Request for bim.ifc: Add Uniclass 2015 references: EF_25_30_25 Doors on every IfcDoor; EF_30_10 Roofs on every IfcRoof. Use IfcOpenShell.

First a look at what the model holds.

```python
import ifcopenshell

model = ifcopenshell.open("bim.ifc")
print(model.schema)
print("classifications:", [c.Name for c in model.by_type("IfcClassification")])
for ifc_class in ("IfcDoor", "IfcRoof", "IfcStair", "IfcWall", "IfcWindow"):
    print(ifc_class, len(model.by_type(ifc_class)))
```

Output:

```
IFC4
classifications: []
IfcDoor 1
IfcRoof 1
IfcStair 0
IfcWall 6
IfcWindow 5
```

```python
import ifcopenshell
import ifcopenshell.api.classification

model = ifcopenshell.open("bim.ifc")

system = ifcopenshell.api.classification.add_classification(model, classification="Uniclass 2015")

codes = {
    "IfcDoor": ("EF_25_30_25", "Doors"),
    "IfcRoof": ("EF_30_10", "Roofs"),
}
for ifc_class, (code, name) in codes.items():
    products = model.by_type(ifc_class)
    ifcopenshell.api.classification.add_reference(
        model, products=products, classification=system, identification=code, name=name
    )
    print(code, len(products))

model.write("bim_edited.ifc")
```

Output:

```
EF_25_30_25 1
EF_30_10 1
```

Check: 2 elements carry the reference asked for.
